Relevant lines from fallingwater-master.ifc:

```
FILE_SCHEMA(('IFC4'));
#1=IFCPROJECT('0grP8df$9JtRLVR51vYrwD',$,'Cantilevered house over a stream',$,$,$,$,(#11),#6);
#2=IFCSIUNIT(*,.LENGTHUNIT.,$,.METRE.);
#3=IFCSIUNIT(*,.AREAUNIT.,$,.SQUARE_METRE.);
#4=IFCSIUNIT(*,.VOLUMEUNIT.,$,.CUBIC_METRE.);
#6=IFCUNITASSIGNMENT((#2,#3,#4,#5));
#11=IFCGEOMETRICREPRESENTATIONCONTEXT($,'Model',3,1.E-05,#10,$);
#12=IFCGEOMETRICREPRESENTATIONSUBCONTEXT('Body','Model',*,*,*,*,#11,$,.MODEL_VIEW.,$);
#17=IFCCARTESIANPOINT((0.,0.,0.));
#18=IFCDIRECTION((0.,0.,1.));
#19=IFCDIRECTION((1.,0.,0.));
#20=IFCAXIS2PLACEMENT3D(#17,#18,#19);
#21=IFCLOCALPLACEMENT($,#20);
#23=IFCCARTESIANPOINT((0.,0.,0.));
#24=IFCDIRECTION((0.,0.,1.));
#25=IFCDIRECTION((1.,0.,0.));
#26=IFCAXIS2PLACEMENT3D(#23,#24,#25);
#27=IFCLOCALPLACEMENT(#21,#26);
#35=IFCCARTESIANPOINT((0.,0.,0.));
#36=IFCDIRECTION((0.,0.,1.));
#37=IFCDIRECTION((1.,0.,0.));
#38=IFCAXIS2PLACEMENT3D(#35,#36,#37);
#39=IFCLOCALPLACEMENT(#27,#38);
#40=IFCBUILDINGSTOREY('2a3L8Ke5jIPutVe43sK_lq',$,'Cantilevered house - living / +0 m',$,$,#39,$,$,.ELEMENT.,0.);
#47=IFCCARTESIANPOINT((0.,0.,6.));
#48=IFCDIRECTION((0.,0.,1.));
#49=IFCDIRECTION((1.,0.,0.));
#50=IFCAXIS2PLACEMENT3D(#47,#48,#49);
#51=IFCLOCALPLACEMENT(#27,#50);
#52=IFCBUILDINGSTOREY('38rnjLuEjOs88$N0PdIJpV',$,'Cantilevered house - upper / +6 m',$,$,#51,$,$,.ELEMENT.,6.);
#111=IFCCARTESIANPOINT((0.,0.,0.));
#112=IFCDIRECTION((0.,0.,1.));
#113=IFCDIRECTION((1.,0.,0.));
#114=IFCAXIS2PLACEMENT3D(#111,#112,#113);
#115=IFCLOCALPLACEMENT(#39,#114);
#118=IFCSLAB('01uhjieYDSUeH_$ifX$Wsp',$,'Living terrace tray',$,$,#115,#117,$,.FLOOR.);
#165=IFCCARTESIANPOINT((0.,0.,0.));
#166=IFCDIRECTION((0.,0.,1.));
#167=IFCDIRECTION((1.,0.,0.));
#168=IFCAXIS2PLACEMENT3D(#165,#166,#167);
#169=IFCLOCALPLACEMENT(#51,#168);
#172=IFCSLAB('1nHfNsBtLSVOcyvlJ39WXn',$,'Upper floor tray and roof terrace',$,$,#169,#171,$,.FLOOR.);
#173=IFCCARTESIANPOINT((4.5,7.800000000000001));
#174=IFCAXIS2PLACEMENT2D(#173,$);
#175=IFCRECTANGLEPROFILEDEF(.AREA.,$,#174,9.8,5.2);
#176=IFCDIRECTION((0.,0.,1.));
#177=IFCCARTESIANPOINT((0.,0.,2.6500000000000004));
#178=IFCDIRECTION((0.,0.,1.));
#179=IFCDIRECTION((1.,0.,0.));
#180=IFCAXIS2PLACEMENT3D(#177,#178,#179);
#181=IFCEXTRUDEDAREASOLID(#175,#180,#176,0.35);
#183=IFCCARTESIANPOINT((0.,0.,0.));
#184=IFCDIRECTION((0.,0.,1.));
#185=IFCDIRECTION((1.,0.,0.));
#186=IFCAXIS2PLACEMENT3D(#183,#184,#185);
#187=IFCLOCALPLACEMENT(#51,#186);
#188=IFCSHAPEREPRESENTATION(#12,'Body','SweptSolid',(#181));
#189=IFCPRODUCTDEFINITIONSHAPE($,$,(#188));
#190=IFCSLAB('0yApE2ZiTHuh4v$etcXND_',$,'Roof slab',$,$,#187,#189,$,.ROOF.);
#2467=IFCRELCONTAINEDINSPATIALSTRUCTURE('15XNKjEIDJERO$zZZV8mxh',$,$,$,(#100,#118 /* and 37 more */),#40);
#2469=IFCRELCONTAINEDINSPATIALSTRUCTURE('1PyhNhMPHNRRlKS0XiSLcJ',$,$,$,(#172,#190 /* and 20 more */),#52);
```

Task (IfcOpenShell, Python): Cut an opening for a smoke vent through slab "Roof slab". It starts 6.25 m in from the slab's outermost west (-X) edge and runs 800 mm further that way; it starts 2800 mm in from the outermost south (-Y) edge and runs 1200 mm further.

```python
import numpy as np
import ifcopenshell
import ifcopenshell.api.feature
import ifcopenshell.api.geometry
import ifcopenshell.api.root
import ifcopenshell.geom
import ifcopenshell.util.placement
import ifcopenshell.util.representation
import ifcopenshell.util.shape
import ifcopenshell.util.unit

model = ifcopenshell.open("fallingwater-master.ifc")
unit_scale = ifcopenshell.util.unit.calculate_unit_scale(model)
settings = ifcopenshell.geom.settings()


def volume(element):
    """Net volume in cubic metres, openings subtracted."""
    shape = ifcopenshell.geom.create_shape(settings, element)
    return ifcopenshell.util.shape.get_volume(shape.geometry)


slab = model.by_guid("0yApE2ZiTHuh4v$etcXND_")
before = volume(slab)

# Extent in the slab's own axes, in metres. The edges named are its -X and -Y sides.
slab_shape = ifcopenshell.geom.create_shape(settings, slab)
vertices = ifcopenshell.util.shape.get_vertices(slab_shape.geometry)
x_min, y_min, bottom = vertices.min(axis=0)
top = vertices[:, 2].max()

opening = ifcopenshell.api.root.create_entity(model, ifc_class="IfcOpeningElement", name="Smoke vent opening", predefined_type="OPENING")
context = ifcopenshell.util.representation.get_context(model, "Model", "Body", "MODEL_VIEW")
width, depth = 0.8, 1.2
outline = [(0.0, 0.0), (width, 0.0), (width, depth), (0.0, depth), (0.0, 0.0)]
# Overshoot both faces by 50 mm so the cut is clean.
shape = ifcopenshell.api.geometry.add_slab_representation(
    model, context=context, depth=top - bottom + 0.1, polyline=outline
)
ifcopenshell.api.geometry.assign_representation(model, product=opening, representation=shape)

matrix = ifcopenshell.util.placement.get_local_placement(slab.ObjectPlacement)
matrix[:, 3] = matrix @ np.append(np.array([x_min + 6.25, y_min + 2.8, bottom - 0.05]) / unit_scale, 1.0)
ifcopenshell.api.geometry.edit_object_placement(model, product=opening, matrix=matrix, is_si=False)
ifcopenshell.api.feature.add_feature(model, feature=opening, element=slab)

after = volume(slab)

print(f"slab volume {before:.3f} -> {after:.3f} m3")

model.write("fallingwater-master_edited.ifc")
```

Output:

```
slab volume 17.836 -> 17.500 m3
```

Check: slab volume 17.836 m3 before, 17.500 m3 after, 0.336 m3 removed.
